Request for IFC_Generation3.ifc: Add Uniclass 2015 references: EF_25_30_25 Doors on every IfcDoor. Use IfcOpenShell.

First a look at what the model holds.

```python
import ifcopenshell

model = ifcopenshell.open("IFC_Generation3.ifc")
print(model.schema)
print("classifications:", [c.Name for c in model.by_type("IfcClassification")])
for ifc_class in ("IfcDoor", "IfcRoof", "IfcStair", "IfcWall", "IfcWindow"):
    print(ifc_class, len(model.by_type(ifc_class)))
```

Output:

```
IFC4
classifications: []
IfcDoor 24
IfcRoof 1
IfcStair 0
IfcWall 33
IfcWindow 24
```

```python
import ifcopenshell
import ifcopenshell.api.classification

model = ifcopenshell.open("IFC_Generation3.ifc")

system = ifcopenshell.api.classification.add_classification(model, classification="Uniclass 2015")

codes = {
    "IfcDoor": ("EF_25_30_25", "Doors"),
}
for ifc_class, (code, name) in codes.items():
    products = model.by_type(ifc_class)
    ifcopenshell.api.classification.add_reference(
        model, products=products, classification=system, identification=code, name=name
    )
    print(code, len(products))

model.write("IFC_Generation3_rev.ifc")
```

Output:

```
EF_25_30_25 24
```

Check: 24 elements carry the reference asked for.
